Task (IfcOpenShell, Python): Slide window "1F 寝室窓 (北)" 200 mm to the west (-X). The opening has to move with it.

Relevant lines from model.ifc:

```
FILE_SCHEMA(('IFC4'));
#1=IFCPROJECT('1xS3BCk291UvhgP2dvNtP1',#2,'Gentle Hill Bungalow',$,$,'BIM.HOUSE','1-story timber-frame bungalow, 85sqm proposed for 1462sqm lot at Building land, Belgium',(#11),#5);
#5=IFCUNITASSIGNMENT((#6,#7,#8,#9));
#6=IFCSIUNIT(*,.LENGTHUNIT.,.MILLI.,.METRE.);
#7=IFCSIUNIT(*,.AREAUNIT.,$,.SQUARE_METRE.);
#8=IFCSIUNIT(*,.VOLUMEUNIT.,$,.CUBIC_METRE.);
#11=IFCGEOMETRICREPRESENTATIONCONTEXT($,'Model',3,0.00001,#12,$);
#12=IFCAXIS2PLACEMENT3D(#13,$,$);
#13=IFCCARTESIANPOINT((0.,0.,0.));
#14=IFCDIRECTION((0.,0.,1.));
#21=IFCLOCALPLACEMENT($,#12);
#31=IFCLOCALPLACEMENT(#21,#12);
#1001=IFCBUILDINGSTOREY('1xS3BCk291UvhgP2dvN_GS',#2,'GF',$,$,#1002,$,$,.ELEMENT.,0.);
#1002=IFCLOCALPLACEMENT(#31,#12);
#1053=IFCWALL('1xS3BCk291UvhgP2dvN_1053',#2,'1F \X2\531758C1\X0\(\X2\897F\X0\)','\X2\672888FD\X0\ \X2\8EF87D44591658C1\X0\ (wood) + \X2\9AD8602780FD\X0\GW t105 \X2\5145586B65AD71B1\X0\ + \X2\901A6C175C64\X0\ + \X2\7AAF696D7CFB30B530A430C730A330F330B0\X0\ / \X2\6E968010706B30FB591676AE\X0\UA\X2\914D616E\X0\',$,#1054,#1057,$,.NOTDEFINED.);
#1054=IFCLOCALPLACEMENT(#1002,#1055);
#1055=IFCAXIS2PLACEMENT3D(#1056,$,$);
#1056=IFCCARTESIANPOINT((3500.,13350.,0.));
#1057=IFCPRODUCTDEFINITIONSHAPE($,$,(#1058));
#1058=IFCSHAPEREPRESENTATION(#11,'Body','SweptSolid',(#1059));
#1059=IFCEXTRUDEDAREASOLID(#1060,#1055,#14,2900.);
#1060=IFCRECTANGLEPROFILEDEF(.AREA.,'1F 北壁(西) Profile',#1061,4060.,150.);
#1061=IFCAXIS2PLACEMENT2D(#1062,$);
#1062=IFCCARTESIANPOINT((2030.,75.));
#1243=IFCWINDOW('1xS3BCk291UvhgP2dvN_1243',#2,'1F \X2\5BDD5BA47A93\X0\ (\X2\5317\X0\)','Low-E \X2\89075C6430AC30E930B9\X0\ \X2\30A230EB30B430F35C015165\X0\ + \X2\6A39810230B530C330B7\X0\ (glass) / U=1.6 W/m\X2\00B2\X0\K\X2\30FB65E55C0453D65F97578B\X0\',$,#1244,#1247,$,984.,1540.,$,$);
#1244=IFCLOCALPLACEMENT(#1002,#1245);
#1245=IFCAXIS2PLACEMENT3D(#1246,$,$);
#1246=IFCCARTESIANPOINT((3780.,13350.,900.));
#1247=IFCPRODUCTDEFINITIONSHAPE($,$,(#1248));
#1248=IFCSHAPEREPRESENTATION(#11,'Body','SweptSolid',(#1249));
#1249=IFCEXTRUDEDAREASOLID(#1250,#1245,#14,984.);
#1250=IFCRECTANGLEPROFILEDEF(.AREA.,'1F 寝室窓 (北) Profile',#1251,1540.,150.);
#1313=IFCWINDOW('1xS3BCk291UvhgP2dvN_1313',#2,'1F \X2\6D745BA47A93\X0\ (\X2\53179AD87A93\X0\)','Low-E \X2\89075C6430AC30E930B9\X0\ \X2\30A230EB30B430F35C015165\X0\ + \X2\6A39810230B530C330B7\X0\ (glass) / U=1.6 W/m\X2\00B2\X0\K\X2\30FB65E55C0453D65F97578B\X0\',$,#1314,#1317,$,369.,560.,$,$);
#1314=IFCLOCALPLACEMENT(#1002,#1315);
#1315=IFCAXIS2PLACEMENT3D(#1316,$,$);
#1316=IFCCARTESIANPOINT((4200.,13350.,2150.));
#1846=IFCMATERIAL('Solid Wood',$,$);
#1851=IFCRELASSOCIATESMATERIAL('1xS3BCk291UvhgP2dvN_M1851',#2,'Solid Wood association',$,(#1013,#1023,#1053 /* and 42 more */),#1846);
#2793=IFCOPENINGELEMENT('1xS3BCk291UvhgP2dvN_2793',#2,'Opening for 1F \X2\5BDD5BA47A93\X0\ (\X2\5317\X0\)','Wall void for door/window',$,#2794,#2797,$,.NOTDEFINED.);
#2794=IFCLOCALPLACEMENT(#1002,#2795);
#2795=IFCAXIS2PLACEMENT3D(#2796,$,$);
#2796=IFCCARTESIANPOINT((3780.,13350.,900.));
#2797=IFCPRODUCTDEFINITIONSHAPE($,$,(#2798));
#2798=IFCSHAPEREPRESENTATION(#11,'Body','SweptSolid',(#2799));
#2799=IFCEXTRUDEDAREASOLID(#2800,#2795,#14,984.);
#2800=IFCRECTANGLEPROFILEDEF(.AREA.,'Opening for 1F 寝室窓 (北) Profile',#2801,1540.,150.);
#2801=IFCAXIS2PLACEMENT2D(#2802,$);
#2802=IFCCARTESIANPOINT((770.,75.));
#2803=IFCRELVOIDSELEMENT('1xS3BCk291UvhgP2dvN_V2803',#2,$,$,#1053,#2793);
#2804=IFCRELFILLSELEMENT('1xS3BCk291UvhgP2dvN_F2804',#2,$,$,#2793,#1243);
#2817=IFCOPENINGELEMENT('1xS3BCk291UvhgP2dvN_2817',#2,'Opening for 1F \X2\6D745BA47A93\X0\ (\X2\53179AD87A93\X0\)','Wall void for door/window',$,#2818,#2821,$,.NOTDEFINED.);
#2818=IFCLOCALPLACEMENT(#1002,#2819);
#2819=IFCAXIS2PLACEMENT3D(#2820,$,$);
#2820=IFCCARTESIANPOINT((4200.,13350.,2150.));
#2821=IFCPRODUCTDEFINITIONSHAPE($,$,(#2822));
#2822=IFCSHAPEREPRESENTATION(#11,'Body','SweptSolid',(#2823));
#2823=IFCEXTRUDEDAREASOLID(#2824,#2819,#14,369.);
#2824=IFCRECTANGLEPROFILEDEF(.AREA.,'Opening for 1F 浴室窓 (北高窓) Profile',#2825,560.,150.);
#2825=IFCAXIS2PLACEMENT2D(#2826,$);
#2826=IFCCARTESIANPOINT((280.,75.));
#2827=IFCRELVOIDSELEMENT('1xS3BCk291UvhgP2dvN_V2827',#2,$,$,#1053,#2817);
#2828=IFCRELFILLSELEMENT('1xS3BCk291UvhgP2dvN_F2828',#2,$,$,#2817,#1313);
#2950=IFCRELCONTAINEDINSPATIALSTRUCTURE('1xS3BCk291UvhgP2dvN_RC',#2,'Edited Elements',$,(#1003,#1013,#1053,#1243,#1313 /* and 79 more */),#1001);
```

```python
import ifcopenshell
import ifcopenshell.api.geometry
import ifcopenshell.util.placement

model = ifcopenshell.open("model.ifc")

window = model.by_guid("1xS3BCk291UvhgP2dvN_1243")
opening = window.FillsVoids[0].RelatingOpeningElement
wall = opening.VoidsElements[0].RelatingBuildingElement

wall_matrix = ifcopenshell.util.placement.get_local_placement(wall.ObjectPlacement)
shift = wall_matrix[:3, 0] * -200.0
before = ifcopenshell.util.placement.get_local_placement(window.ObjectPlacement)[:3, 3].copy()

# The window is not placed relative to its opening, so move both.
for product in (opening, window):
    matrix = ifcopenshell.util.placement.get_local_placement(product.ObjectPlacement)
    matrix[:3, 3] += shift
    ifcopenshell.api.geometry.edit_object_placement(model, product=product, matrix=matrix, is_si=False)

after = ifcopenshell.util.placement.get_local_placement(window.ObjectPlacement)[:3, 3]
print("window moved by", (after - before).round(3) + 0.0)

model.write("model-out.ifc")
```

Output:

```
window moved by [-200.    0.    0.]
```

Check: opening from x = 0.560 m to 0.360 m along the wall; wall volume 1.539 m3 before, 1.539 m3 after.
